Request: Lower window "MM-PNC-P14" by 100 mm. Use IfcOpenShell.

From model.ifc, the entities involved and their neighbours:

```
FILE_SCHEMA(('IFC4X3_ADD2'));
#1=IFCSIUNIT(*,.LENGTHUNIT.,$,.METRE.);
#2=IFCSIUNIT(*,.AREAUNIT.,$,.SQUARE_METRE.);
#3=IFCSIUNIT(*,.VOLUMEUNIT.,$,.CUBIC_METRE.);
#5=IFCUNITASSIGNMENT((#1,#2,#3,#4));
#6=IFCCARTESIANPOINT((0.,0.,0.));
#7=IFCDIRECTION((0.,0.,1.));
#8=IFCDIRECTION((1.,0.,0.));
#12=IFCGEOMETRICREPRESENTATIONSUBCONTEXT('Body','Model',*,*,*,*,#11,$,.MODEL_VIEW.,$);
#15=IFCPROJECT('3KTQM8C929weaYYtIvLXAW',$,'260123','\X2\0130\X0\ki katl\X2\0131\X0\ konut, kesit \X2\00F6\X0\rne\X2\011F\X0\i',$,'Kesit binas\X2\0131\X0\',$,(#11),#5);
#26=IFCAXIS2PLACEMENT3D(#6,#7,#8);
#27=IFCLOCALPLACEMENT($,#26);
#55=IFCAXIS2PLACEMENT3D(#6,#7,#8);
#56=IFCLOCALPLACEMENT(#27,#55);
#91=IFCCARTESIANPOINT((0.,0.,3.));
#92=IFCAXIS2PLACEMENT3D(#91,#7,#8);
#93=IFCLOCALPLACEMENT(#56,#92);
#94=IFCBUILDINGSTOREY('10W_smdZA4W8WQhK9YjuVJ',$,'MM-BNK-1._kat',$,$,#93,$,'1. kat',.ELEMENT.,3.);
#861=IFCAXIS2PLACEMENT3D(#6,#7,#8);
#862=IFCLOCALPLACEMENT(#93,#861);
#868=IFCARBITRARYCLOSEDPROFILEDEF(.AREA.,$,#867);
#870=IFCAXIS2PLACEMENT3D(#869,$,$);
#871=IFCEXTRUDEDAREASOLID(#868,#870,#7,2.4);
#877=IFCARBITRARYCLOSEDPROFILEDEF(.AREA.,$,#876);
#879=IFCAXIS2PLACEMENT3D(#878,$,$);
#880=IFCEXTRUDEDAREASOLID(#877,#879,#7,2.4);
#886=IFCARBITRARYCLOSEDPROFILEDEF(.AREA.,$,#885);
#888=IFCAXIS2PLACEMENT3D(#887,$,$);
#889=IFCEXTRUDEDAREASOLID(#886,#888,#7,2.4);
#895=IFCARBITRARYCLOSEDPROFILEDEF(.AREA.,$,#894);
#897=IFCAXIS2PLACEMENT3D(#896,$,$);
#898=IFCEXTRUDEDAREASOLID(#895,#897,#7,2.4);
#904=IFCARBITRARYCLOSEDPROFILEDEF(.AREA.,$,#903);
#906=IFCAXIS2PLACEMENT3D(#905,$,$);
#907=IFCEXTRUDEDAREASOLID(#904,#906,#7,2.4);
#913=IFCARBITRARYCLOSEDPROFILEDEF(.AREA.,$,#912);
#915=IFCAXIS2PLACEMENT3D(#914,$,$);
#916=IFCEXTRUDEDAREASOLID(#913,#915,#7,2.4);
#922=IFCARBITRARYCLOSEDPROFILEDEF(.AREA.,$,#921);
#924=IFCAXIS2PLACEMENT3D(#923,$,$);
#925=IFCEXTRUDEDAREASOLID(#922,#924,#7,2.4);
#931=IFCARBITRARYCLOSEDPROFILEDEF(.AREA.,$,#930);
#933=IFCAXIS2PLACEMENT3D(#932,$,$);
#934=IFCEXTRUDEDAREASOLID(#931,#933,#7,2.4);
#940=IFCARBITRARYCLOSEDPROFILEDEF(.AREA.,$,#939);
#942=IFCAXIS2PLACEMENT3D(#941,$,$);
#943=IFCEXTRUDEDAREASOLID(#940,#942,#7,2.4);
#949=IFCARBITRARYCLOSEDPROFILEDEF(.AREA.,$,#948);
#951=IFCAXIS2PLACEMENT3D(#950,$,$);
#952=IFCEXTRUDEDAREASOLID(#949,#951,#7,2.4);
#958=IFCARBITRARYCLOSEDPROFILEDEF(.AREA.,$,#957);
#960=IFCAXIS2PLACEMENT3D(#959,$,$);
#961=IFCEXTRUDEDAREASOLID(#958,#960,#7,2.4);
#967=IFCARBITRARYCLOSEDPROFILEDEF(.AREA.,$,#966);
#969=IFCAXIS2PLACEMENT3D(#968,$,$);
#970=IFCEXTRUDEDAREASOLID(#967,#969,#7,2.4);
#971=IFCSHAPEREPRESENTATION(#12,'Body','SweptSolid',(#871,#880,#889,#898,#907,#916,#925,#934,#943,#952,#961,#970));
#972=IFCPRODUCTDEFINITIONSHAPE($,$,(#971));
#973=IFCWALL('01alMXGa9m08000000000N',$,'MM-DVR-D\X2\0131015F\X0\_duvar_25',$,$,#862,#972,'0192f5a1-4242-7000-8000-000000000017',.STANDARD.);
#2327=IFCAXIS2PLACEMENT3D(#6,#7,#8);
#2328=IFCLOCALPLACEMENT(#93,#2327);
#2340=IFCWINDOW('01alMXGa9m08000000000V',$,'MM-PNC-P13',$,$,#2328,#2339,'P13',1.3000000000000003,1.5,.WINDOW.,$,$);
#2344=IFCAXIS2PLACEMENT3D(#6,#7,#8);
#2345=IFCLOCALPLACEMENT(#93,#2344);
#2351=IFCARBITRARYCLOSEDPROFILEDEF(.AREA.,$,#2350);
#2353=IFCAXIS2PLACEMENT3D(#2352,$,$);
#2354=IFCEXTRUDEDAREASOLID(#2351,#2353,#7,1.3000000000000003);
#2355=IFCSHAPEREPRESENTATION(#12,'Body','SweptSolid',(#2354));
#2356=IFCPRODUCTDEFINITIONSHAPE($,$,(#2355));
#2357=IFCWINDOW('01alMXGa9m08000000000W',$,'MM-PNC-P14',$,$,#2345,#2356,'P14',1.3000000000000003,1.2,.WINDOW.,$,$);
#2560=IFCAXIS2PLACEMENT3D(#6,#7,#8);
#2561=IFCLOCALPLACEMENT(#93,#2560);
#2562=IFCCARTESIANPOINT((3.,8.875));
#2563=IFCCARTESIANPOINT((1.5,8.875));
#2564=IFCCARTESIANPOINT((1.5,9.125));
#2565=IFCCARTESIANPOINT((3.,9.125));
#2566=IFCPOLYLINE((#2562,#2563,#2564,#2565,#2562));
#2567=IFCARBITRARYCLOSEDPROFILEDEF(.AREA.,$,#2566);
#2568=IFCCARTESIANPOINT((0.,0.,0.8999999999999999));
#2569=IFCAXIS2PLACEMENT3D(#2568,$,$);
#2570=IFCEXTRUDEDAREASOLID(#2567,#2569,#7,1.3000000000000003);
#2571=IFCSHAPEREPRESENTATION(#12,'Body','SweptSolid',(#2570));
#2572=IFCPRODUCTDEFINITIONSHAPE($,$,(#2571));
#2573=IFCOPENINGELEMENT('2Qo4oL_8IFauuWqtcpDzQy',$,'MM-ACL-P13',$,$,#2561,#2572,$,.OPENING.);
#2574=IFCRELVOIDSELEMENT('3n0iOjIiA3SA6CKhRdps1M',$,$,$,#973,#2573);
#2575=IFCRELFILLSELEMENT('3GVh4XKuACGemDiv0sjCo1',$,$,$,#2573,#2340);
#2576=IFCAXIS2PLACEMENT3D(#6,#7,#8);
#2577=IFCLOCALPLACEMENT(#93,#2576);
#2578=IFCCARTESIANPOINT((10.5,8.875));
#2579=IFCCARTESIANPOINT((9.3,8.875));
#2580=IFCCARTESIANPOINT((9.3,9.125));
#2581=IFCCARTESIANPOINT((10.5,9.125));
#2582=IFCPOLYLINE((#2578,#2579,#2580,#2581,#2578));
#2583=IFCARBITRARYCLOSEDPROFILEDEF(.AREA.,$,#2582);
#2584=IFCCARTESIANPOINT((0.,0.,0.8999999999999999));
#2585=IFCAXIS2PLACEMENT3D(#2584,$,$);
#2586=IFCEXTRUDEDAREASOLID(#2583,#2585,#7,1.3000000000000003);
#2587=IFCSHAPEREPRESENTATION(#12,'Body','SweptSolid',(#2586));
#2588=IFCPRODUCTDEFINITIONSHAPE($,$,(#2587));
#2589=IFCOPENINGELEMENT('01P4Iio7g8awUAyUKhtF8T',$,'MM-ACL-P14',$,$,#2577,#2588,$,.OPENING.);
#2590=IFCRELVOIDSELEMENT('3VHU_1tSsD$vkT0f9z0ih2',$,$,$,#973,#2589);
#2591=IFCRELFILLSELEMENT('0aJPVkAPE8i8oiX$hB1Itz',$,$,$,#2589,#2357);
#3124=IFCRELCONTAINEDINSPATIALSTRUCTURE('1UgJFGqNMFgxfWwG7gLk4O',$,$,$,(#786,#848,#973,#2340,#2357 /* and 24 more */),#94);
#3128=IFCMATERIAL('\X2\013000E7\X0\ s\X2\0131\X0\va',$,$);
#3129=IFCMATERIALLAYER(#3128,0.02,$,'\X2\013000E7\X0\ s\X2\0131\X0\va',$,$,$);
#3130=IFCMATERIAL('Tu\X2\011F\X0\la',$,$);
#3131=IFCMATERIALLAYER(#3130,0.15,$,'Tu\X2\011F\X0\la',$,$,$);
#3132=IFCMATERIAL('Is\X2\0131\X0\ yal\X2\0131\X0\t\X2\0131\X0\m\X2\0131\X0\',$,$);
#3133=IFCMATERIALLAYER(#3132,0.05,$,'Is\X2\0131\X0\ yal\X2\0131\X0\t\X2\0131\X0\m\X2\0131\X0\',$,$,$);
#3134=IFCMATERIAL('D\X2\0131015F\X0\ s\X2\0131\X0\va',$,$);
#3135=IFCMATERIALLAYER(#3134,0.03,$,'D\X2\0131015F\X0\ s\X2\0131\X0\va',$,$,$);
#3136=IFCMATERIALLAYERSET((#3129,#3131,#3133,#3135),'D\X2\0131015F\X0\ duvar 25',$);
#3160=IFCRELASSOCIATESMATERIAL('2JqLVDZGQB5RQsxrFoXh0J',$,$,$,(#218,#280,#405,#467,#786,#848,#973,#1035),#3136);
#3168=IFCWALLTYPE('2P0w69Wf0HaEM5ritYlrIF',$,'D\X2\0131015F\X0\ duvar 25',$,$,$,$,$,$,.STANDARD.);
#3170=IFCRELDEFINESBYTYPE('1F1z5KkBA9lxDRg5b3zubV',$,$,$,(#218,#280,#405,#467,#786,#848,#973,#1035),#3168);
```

```python
import numpy as np
import ifcopenshell
import ifcopenshell.api.geometry
import ifcopenshell.util.placement
import ifcopenshell.util.unit

model = ifcopenshell.open("model.ifc")
unit_scale = ifcopenshell.util.unit.calculate_unit_scale(model)

window = model.by_guid("01alMXGa9m08000000000W")
opening = window.FillsVoids[0].RelatingOpeningElement
dz = -0.1

shift = np.array([0.0, 0.0, dz])
# The window is not placed relative to its opening, so move both.
for product in (opening, window):
    matrix = ifcopenshell.util.placement.get_local_placement(product.ObjectPlacement)
    matrix[:3, 3] += shift
    ifcopenshell.api.geometry.edit_object_placement(model, product=product, matrix=matrix, is_si=False)

print(f"moved by {dz * unit_scale:+.3f} m")

model.write("model-out.ifc")
```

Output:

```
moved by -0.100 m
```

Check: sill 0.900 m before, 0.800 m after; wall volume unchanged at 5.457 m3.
